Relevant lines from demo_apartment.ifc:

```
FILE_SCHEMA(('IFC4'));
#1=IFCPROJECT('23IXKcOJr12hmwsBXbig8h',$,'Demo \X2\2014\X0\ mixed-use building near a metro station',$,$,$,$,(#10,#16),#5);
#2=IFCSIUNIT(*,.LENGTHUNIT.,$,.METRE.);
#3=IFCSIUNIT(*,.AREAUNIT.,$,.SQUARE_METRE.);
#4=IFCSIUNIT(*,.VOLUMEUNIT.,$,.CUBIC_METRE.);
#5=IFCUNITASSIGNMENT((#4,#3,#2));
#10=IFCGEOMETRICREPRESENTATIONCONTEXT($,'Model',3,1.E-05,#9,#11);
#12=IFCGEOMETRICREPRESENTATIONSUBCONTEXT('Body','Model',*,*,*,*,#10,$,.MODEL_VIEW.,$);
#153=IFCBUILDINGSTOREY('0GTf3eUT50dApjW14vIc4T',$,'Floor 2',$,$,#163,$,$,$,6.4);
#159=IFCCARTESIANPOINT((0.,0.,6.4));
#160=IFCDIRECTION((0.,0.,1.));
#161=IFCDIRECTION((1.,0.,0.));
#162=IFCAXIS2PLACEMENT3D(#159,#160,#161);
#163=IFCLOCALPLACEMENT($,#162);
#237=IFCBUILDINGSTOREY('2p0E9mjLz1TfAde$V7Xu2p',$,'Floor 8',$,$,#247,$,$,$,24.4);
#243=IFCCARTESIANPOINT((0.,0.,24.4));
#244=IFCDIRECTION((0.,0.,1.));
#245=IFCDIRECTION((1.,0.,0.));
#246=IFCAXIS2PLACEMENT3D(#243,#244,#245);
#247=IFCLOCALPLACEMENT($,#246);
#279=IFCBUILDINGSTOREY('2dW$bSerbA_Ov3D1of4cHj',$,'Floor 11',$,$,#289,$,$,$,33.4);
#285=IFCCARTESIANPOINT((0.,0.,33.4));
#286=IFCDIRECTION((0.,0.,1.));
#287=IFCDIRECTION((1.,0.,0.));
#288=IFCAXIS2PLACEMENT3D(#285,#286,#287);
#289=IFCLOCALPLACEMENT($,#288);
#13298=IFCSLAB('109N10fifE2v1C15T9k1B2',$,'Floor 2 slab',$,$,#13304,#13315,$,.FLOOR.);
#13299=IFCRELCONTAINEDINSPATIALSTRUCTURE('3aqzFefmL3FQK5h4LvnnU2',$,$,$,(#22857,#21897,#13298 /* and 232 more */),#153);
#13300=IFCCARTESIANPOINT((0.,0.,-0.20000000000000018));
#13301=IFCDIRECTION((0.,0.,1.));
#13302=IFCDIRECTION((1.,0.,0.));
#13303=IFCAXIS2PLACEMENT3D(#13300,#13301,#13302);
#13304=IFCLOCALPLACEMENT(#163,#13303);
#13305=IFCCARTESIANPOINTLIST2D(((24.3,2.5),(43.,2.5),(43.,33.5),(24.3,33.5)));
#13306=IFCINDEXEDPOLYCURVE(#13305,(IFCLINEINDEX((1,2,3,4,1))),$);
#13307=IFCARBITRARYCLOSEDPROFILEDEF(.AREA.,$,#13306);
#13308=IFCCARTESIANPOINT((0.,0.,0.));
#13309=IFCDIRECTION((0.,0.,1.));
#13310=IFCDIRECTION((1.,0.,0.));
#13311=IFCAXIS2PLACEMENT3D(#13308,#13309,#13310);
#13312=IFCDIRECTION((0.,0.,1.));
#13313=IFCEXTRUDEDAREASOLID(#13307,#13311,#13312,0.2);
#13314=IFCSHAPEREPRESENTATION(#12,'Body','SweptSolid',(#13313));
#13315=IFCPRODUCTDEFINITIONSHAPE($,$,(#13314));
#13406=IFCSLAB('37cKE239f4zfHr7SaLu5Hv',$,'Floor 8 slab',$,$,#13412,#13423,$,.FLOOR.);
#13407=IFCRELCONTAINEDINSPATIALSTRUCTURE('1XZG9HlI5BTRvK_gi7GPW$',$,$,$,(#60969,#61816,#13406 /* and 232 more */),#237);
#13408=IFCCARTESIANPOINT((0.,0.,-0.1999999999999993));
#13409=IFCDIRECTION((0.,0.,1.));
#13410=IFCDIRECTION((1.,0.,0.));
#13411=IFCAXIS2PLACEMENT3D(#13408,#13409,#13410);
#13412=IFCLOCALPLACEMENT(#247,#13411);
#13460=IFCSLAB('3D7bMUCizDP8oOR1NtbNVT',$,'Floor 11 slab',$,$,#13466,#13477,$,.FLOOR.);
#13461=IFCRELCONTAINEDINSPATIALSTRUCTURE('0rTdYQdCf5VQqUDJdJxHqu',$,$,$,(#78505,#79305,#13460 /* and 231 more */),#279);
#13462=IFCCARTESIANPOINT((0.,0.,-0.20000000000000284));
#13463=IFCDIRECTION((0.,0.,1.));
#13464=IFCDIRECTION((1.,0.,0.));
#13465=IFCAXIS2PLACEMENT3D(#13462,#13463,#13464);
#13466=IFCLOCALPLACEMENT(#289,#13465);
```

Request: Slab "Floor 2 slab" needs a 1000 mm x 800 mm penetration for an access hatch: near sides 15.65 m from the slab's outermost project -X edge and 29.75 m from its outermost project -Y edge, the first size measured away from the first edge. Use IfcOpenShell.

```python
import numpy as np
import ifcopenshell
import ifcopenshell.api.feature
import ifcopenshell.api.geometry
import ifcopenshell.api.root
import ifcopenshell.geom
import ifcopenshell.util.placement
import ifcopenshell.util.representation
import ifcopenshell.util.shape
import ifcopenshell.util.unit

model = ifcopenshell.open("demo_apartment.ifc")
unit_scale = ifcopenshell.util.unit.calculate_unit_scale(model)
settings = ifcopenshell.geom.settings()


def volume(element):
    """Net volume in cubic metres, openings subtracted."""
    shape = ifcopenshell.geom.create_shape(settings, element)
    return ifcopenshell.util.shape.get_volume(shape.geometry)


slab = model.by_guid("109N10fifE2v1C15T9k1B2")
before = volume(slab)

# Extent in the slab's own axes, in metres. The edges named are its -X and -Y sides.
slab_shape = ifcopenshell.geom.create_shape(settings, slab)
vertices = ifcopenshell.util.shape.get_vertices(slab_shape.geometry)
x_min, y_min, bottom = vertices.min(axis=0)
top = vertices[:, 2].max()

opening = ifcopenshell.api.root.create_entity(model, ifc_class="IfcOpeningElement", name="Access hatch opening", predefined_type="OPENING")
context = ifcopenshell.util.representation.get_context(model, "Model", "Body", "MODEL_VIEW")
width, depth = 1, 0.8
outline = [(0.0, 0.0), (width, 0.0), (width, depth), (0.0, depth), (0.0, 0.0)]
# Overshoot both faces by 50 mm so the cut is clean.
shape = ifcopenshell.api.geometry.add_slab_representation(
    model, context=context, depth=top - bottom + 0.1, polyline=outline
)
ifcopenshell.api.geometry.assign_representation(model, product=opening, representation=shape)

matrix = ifcopenshell.util.placement.get_local_placement(slab.ObjectPlacement)
matrix[:, 3] = matrix @ np.append(np.array([x_min + 15.65, y_min + 29.75, bottom - 0.05]) / unit_scale, 1.0)
ifcopenshell.api.geometry.edit_object_placement(model, product=opening, matrix=matrix, is_si=False)
ifcopenshell.api.feature.add_feature(model, feature=opening, element=slab)

after = volume(slab)

print(f"slab volume {before:.3f} -> {after:.3f} m3")

model.write("demo_apartment_v2.ifc")
```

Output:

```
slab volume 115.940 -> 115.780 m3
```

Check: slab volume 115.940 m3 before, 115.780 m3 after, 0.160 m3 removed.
